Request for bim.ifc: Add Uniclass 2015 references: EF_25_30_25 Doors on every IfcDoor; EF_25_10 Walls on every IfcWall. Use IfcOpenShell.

First a look at what the model holds.

```python
import ifcopenshell

model = ifcopenshell.open("bim.ifc")
print(model.schema)
print("classifications:", [c.Name for c in model.by_type("IfcClassification")])
for ifc_class in ("IfcDoor", "IfcRoof", "IfcStair", "IfcWall", "IfcWindow"):
    print(ifc_class, len(model.by_type(ifc_class)))
```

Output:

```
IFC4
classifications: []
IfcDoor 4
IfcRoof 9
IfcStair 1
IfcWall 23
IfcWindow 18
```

```python
import ifcopenshell
import ifcopenshell.api.classification

model = ifcopenshell.open("bim.ifc")

system = ifcopenshell.api.classification.add_classification(model, classification="Uniclass 2015")

codes = {
    "IfcDoor": ("EF_25_30_25", "Doors"),
    "IfcWall": ("EF_25_10", "Walls"),
}
for ifc_class, (code, name) in codes.items():
    products = model.by_type(ifc_class)
    ifcopenshell.api.classification.add_reference(
        model, products=products, classification=system, identification=code, name=name
    )
    print(code, len(products))

model.write("bim_edited.ifc")
```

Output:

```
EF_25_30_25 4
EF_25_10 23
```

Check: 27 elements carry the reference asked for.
